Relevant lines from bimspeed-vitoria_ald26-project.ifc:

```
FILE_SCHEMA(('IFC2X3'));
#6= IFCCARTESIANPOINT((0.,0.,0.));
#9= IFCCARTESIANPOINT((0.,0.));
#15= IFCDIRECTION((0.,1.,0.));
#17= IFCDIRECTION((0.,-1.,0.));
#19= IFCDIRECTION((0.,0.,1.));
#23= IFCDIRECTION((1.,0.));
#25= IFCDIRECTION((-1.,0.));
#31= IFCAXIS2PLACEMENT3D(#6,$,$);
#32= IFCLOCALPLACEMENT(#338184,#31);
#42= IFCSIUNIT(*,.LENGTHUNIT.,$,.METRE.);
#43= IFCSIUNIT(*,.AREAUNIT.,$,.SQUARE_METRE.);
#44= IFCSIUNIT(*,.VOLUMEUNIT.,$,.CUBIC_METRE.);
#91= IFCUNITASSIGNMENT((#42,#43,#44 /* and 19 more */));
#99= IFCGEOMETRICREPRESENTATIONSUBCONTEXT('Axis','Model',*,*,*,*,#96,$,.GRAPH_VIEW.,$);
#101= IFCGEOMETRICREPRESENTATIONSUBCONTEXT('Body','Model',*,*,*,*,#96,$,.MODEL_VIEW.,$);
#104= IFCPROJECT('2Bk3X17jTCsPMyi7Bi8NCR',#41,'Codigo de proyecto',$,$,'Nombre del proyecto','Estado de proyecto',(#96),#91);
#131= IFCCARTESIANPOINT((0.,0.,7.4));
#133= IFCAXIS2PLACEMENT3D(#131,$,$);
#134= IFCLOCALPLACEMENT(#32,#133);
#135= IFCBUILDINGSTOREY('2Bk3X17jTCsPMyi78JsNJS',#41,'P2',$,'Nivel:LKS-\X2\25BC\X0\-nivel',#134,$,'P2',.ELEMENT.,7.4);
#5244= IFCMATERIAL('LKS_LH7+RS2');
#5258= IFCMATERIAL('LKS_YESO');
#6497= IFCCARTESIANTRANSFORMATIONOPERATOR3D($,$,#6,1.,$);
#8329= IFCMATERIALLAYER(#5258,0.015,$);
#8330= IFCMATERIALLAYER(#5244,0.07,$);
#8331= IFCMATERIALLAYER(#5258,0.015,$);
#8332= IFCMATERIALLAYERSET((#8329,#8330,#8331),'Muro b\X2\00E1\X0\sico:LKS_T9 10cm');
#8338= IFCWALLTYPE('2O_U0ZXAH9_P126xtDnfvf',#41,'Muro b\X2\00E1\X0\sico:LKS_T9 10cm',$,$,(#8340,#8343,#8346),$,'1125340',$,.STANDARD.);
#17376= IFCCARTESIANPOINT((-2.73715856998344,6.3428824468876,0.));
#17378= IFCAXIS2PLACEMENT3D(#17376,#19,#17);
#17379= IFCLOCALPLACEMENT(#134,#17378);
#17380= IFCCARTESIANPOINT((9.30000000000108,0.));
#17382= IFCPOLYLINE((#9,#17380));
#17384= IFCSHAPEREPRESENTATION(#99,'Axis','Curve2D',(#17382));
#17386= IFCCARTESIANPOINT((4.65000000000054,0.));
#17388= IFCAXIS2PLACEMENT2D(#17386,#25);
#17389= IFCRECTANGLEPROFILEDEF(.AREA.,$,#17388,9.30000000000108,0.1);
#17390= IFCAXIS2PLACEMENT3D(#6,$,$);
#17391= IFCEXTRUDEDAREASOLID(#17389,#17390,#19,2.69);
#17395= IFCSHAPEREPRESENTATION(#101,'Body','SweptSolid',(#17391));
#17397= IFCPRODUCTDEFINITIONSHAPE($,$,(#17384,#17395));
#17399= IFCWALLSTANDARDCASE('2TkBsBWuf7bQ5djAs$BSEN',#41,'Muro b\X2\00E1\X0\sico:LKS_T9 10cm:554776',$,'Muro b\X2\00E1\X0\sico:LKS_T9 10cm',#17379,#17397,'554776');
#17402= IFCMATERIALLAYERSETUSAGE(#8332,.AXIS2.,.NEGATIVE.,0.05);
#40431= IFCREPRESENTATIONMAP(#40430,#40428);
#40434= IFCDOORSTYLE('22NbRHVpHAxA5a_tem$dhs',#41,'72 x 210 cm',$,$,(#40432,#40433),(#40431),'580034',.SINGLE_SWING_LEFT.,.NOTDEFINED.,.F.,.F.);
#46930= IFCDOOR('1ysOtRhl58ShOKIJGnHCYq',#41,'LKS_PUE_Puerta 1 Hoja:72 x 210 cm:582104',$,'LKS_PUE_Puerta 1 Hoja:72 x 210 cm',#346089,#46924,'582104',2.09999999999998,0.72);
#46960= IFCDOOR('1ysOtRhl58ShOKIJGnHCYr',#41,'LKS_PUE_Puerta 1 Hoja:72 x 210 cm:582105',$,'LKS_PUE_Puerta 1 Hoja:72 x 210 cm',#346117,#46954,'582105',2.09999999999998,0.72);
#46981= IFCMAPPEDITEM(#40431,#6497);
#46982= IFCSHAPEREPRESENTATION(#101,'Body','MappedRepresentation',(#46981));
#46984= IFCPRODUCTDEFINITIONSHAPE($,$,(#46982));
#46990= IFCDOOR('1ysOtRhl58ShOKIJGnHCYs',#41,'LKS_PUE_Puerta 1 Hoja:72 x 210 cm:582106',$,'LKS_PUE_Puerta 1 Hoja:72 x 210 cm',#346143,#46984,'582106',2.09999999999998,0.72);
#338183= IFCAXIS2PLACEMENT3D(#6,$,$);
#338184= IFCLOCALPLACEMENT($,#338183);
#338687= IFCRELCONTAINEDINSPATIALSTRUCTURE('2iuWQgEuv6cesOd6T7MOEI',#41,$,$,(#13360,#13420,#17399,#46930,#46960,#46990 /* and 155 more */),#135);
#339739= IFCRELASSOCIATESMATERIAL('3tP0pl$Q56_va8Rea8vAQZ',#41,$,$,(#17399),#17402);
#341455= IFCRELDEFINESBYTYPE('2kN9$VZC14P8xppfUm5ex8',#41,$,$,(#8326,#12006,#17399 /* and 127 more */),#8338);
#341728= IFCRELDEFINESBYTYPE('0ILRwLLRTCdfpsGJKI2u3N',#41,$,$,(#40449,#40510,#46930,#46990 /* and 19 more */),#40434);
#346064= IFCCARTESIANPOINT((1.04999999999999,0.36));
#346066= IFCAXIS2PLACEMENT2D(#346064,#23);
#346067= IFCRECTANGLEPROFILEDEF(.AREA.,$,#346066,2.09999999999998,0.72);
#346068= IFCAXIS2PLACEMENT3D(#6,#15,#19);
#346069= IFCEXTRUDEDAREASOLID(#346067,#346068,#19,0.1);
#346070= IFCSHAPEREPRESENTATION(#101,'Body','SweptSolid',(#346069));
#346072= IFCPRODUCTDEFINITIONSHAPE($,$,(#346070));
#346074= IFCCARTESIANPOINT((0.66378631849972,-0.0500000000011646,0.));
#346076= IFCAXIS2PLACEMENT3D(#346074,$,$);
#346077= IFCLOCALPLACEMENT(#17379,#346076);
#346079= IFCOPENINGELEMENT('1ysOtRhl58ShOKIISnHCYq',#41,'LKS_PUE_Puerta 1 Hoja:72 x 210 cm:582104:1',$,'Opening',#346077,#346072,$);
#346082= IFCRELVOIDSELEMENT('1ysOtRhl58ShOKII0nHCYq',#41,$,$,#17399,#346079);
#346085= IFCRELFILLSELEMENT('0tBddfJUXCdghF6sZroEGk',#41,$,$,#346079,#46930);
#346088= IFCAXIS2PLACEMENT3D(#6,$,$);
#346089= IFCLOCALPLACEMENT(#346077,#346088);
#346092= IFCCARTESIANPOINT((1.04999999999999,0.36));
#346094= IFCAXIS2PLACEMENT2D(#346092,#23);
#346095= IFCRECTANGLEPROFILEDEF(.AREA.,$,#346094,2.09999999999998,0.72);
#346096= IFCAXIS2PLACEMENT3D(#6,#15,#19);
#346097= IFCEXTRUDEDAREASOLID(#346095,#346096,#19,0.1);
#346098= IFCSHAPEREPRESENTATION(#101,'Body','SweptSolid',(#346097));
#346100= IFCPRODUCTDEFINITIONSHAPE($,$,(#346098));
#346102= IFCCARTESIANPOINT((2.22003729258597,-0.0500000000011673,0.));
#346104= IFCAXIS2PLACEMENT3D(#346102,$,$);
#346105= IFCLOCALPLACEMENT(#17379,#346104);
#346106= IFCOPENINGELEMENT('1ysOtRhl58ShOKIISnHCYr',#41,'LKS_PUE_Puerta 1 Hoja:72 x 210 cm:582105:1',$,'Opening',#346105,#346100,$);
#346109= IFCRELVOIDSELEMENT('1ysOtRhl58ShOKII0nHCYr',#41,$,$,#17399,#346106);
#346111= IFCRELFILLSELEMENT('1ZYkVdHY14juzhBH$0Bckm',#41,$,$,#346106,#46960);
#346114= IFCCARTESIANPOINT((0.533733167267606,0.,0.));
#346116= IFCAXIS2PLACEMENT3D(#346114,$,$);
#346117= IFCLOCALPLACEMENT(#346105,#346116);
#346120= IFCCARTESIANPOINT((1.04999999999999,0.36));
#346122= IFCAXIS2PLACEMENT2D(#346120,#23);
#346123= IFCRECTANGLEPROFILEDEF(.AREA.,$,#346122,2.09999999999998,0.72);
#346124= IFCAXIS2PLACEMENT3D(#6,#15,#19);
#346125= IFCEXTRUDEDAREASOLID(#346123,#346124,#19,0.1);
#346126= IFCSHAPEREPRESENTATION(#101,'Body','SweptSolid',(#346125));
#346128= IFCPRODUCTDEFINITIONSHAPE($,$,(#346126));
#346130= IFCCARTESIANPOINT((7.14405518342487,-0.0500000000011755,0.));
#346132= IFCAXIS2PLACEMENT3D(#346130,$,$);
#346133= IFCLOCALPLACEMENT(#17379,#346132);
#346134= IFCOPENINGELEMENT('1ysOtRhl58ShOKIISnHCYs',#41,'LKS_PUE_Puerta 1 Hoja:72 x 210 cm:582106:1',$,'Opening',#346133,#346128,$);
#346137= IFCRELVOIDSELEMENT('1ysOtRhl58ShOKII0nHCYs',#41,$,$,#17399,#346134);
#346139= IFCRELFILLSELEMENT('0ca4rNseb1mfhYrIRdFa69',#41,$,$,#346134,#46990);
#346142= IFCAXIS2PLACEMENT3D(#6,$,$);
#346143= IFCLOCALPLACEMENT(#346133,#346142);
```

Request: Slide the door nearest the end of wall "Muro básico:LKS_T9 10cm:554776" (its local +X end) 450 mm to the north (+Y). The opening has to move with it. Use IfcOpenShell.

```python
import ifcopenshell
import ifcopenshell.api.geometry
import ifcopenshell.util.placement
import ifcopenshell.util.unit

model = ifcopenshell.open("bimspeed-vitoria_ald26-project.ifc")
unit_scale = ifcopenshell.util.unit.calculate_unit_scale(model)

door = model.by_guid("1ysOtRhl58ShOKIJGnHCYs")
opening = door.FillsVoids[0].RelatingOpeningElement
wall = opening.VoidsElements[0].RelatingBuildingElement

wall_matrix = ifcopenshell.util.placement.get_local_placement(wall.ObjectPlacement)
shift = wall_matrix[:3, 0] * -0.45 / unit_scale
before = ifcopenshell.util.placement.get_local_placement(door.ObjectPlacement)[:3, 3].copy()

# The door is placed relative to its opening, so it follows when the opening moves.
matrix = ifcopenshell.util.placement.get_local_placement(opening.ObjectPlacement)
matrix[:3, 3] += shift
ifcopenshell.api.geometry.edit_object_placement(
    model, product=opening, matrix=matrix, is_si=False, should_transform_children=True
)

after = ifcopenshell.util.placement.get_local_placement(door.ObjectPlacement)[:3, 3]
print("door moved by", (after - before).round(3) + 0.0)

model.write("bimspeed-vitoria_ald26-project_v2.ifc")
```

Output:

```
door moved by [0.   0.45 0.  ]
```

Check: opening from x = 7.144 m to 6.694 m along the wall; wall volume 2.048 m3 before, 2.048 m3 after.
